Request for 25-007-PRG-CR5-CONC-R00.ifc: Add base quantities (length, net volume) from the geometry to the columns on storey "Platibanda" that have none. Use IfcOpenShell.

First a look at what the model holds.

```python
import ifcopenshell
import ifcopenshell.util.element
import ifcopenshell.util.unit

model = ifcopenshell.open("25-007-PRG-CR5-CONC-R00.ifc")
print(model.schema)
for unit_type in ("LENGTHUNIT", "AREAUNIT", "VOLUMEUNIT"):
    print(unit_type, ifcopenshell.util.unit.calculate_unit_scale(model, unit_type))
storey = next(s for s in model.by_type("IfcBuildingStorey") if s.Name == "Platibanda")
columns = [e for e in ifcopenshell.util.element.get_decomposition(storey) if e.is_a("IfcColumn")]
for e in sorted(columns, key=lambda e: e.id()):
    print(e.id(), e.is_a(), e.Name, list(ifcopenshell.util.element.get_psets(e, qtos_only=True)), sep=" | ")
```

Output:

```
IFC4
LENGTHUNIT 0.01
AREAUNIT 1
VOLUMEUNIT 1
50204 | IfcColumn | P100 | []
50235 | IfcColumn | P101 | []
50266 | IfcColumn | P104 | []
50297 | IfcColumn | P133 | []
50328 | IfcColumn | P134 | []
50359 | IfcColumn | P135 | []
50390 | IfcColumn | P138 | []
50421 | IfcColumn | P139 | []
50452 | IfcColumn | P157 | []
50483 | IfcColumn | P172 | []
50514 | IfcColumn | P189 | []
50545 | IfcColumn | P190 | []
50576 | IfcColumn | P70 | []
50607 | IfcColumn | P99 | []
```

```python
import ifcopenshell
import ifcopenshell.api.pset
import ifcopenshell.geom
import ifcopenshell.util.element
import ifcopenshell.util.shape
import ifcopenshell.util.unit

model = ifcopenshell.open("25-007-PRG-CR5-CONC-R00.ifc")
unit_scale = ifcopenshell.util.unit.calculate_unit_scale(model)
volume_scale = ifcopenshell.util.unit.calculate_unit_scale(model, "VOLUMEUNIT")
settings = ifcopenshell.geom.settings()

storey = next(s for s in model.by_type("IfcBuildingStorey") if s.Name == "Platibanda")
columns = [e for e in ifcopenshell.util.element.get_decomposition(storey) if e.is_a("IfcColumn")]

for e in sorted(columns, key=lambda e: e.id()):
    if ifcopenshell.util.element.get_psets(e, qtos_only=True, should_inherit=False):
        continue
    # Geometry comes back in metres, in the element's own axes.
    shape = ifcopenshell.geom.create_shape(settings, e)
    values = {
        "Length": ifcopenshell.util.shape.get_z(shape.geometry) / unit_scale,
        "NetVolume": ifcopenshell.util.shape.get_volume(shape.geometry) / volume_scale,
    }
    qto = ifcopenshell.api.pset.add_qto(model, product=e, name="Qto_ColumnBaseQuantities")
    ifcopenshell.api.pset.edit_qto(model, qto=qto, properties=values)
    print(e.id(), {k: round(v, 3) for k, v in values.items()})

model.write("25-007-PRG-CR5-CONC-R00_edited.ifc")
```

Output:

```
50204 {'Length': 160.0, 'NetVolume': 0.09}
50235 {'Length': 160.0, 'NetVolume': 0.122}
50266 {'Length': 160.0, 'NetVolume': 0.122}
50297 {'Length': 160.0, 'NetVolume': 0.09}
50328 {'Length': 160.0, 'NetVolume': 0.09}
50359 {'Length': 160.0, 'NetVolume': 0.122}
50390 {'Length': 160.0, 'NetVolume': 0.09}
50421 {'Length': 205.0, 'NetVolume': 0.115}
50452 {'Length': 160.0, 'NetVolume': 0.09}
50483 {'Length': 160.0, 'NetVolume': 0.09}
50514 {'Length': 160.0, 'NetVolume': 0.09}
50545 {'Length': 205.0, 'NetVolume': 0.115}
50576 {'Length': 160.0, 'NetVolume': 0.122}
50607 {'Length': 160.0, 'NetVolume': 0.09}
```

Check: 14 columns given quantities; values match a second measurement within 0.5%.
